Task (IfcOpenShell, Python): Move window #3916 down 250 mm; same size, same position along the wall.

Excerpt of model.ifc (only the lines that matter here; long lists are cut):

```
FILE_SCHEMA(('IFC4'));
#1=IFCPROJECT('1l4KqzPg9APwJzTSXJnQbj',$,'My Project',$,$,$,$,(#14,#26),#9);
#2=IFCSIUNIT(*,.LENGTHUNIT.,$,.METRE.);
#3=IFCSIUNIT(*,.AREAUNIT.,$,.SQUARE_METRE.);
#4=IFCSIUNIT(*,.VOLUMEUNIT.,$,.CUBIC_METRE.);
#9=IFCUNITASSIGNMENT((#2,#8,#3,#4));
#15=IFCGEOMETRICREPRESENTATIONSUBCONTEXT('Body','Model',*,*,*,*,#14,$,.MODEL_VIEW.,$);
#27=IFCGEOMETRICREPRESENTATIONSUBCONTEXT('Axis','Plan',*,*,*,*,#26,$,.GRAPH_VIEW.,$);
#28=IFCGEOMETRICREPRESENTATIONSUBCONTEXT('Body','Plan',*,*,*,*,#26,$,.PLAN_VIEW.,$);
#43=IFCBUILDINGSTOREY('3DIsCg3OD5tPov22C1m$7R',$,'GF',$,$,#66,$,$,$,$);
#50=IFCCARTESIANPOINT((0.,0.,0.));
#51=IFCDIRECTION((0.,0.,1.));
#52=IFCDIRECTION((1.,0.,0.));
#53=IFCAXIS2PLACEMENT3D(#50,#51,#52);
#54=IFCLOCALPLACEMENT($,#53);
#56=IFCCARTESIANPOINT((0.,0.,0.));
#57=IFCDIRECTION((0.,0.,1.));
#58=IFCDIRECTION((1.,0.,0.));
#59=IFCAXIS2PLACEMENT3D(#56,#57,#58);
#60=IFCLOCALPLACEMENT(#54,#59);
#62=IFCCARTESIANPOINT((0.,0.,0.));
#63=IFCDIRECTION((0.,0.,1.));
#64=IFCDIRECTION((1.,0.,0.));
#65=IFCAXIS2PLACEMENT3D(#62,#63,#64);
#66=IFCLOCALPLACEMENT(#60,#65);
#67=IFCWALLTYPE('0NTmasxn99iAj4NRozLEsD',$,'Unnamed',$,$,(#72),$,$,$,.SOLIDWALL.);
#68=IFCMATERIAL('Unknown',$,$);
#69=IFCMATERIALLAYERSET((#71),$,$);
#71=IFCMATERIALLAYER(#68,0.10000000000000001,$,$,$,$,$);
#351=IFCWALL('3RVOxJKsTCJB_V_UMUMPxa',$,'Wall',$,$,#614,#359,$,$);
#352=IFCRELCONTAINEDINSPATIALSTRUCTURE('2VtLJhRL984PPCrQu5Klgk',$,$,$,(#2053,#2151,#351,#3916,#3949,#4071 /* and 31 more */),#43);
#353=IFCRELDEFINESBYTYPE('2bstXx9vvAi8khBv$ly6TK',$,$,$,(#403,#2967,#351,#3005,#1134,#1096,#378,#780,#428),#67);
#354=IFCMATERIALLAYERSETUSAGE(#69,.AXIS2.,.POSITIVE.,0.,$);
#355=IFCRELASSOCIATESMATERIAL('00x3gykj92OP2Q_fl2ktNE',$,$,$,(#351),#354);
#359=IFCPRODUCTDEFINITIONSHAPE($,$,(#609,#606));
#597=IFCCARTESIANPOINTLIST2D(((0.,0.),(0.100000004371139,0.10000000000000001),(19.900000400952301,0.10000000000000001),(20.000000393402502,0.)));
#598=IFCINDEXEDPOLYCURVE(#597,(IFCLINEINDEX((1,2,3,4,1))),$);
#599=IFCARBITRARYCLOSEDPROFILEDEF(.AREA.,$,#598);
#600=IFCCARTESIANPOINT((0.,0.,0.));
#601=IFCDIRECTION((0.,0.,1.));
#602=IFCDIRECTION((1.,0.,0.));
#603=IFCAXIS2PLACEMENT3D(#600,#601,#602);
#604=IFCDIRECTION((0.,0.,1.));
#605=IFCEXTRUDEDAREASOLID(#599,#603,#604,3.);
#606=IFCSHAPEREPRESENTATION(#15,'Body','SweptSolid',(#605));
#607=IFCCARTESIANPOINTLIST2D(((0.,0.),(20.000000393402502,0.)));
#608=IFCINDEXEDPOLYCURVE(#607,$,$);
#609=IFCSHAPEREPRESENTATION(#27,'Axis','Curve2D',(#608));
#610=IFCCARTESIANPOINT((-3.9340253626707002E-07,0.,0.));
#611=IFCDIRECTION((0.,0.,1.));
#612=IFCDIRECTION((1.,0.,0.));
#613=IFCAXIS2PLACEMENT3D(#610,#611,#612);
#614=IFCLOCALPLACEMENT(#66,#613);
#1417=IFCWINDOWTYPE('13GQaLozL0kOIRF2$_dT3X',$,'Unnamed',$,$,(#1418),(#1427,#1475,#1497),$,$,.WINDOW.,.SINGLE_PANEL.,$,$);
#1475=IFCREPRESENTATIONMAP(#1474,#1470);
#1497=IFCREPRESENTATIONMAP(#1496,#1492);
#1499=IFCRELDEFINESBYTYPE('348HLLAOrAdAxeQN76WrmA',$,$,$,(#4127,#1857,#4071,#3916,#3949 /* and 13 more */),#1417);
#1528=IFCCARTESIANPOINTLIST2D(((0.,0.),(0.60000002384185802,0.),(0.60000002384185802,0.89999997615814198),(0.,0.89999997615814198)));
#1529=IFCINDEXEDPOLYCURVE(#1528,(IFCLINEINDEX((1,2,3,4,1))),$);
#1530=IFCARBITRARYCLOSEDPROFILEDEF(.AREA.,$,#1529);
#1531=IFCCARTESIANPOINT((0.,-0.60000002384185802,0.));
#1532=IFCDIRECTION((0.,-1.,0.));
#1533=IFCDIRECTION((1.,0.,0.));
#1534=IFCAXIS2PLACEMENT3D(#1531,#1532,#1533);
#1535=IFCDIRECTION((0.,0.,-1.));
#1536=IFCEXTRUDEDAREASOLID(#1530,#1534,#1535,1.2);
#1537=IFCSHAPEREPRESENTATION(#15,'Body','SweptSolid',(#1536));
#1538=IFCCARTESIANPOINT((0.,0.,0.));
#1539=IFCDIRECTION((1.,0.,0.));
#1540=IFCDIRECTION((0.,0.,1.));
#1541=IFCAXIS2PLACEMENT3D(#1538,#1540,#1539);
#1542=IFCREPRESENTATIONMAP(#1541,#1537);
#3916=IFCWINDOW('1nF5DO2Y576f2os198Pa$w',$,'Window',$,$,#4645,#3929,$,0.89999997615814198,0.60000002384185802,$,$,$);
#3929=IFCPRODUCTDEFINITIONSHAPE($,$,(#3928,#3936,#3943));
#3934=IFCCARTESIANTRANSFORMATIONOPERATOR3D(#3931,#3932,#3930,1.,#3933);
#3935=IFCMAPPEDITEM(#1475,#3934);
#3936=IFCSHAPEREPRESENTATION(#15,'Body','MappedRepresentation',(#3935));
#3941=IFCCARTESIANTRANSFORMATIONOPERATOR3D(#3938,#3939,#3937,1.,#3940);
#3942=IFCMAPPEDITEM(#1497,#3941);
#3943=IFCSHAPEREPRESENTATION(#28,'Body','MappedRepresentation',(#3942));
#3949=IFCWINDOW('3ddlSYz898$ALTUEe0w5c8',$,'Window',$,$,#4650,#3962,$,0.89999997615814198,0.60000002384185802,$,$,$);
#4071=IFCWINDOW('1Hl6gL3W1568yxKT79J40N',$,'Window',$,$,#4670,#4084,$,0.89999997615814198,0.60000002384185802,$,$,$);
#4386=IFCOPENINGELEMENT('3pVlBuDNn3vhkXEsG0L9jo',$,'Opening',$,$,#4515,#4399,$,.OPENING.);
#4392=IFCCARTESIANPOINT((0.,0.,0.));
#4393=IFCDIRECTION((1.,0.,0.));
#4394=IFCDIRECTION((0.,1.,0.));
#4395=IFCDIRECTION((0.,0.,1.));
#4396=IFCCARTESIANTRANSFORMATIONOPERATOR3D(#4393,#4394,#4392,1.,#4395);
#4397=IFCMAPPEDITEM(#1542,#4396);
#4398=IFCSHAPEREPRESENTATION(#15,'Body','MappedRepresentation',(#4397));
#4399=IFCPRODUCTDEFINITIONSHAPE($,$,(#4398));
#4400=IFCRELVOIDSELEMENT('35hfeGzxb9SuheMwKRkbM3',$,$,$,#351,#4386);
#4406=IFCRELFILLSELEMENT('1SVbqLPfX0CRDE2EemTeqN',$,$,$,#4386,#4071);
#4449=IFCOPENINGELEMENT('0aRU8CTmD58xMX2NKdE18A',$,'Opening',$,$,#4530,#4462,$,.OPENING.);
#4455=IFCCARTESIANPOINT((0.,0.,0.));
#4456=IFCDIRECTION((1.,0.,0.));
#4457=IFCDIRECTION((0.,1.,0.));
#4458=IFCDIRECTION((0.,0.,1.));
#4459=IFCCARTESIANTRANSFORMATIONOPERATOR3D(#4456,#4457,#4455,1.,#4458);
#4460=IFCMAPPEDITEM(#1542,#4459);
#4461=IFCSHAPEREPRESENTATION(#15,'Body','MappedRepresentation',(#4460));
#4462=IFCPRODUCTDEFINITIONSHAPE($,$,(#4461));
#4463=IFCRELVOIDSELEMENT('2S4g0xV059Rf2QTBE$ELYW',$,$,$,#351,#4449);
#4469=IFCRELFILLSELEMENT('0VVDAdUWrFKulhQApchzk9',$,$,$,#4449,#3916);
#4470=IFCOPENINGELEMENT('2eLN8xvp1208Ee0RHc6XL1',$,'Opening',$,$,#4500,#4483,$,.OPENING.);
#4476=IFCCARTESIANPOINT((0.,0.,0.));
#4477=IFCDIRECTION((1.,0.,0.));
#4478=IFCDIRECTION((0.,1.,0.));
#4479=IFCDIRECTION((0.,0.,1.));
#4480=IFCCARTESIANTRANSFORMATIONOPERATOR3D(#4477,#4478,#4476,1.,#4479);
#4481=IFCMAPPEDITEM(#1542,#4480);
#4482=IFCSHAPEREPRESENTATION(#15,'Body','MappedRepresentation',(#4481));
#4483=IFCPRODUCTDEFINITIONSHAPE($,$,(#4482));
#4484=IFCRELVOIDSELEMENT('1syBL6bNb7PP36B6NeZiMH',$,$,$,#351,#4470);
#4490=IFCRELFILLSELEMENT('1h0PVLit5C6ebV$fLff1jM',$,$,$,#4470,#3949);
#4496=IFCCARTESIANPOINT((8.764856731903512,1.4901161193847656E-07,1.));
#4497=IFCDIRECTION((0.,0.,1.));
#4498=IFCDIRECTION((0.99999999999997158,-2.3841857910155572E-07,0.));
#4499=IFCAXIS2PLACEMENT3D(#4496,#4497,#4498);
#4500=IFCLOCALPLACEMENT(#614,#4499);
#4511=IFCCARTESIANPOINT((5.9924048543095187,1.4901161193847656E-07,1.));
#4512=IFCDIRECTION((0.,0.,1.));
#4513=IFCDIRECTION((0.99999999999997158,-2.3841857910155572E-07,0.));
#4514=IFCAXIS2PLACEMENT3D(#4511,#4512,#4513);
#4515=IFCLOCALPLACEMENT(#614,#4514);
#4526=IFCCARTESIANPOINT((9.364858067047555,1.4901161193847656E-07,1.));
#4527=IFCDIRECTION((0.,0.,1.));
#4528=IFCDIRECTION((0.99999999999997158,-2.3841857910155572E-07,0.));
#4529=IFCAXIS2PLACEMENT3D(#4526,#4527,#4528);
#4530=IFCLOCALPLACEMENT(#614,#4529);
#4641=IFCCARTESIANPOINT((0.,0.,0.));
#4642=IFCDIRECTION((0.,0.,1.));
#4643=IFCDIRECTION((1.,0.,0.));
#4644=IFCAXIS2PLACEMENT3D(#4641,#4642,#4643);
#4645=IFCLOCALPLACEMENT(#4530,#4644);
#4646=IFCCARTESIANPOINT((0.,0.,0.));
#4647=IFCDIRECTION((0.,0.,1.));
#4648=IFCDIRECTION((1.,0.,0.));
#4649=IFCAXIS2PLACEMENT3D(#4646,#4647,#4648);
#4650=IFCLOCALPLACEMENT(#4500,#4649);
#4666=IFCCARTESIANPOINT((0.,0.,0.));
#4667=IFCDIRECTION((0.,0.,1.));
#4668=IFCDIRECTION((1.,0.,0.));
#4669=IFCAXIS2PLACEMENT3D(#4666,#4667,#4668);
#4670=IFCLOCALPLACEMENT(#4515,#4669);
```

```python
import numpy as np
import ifcopenshell
import ifcopenshell.api.geometry
import ifcopenshell.util.placement
import ifcopenshell.util.unit

model = ifcopenshell.open("model.ifc")
unit_scale = ifcopenshell.util.unit.calculate_unit_scale(model)

window = model.by_guid("1nF5DO2Y576f2os198Pa$w")
opening = window.FillsVoids[0].RelatingOpeningElement
dz = -0.25

shift = np.array([0.0, 0.0, dz])
# The window is placed relative to its opening, so it follows when the opening moves.
matrix = ifcopenshell.util.placement.get_local_placement(opening.ObjectPlacement)
matrix[:3, 3] += shift
ifcopenshell.api.geometry.edit_object_placement(
    model, product=opening, matrix=matrix, is_si=False, should_transform_children=True
)

print(f"moved by {dz * unit_scale:+.3f} m")

model.write("model_updated.ifc")
```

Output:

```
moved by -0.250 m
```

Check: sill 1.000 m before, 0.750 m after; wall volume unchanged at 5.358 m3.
